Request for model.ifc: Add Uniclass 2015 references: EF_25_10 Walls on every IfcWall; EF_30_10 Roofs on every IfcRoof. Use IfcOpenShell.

First a look at what the model holds.

```python
import ifcopenshell

model = ifcopenshell.open("model.ifc")
print(model.schema)
print("classifications:", [c.Name for c in model.by_type("IfcClassification")])
for ifc_class in ("IfcDoor", "IfcRoof", "IfcStair", "IfcWall", "IfcWindow"):
    print(ifc_class, len(model.by_type(ifc_class)))
```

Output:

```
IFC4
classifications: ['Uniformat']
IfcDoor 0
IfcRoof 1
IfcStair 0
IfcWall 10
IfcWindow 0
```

```python
import ifcopenshell
import ifcopenshell.api.classification

model = ifcopenshell.open("model.ifc")

system = ifcopenshell.api.classification.add_classification(model, classification="Uniclass 2015")

codes = {
    "IfcWall": ("EF_25_10", "Walls"),
    "IfcRoof": ("EF_30_10", "Roofs"),
}
for ifc_class, (code, name) in codes.items():
    products = model.by_type(ifc_class)
    ifcopenshell.api.classification.add_reference(
        model, products=products, classification=system, identification=code, name=name
    )
    print(code, len(products))

model.write("model_updated.ifc")
```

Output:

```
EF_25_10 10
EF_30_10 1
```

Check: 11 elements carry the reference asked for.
